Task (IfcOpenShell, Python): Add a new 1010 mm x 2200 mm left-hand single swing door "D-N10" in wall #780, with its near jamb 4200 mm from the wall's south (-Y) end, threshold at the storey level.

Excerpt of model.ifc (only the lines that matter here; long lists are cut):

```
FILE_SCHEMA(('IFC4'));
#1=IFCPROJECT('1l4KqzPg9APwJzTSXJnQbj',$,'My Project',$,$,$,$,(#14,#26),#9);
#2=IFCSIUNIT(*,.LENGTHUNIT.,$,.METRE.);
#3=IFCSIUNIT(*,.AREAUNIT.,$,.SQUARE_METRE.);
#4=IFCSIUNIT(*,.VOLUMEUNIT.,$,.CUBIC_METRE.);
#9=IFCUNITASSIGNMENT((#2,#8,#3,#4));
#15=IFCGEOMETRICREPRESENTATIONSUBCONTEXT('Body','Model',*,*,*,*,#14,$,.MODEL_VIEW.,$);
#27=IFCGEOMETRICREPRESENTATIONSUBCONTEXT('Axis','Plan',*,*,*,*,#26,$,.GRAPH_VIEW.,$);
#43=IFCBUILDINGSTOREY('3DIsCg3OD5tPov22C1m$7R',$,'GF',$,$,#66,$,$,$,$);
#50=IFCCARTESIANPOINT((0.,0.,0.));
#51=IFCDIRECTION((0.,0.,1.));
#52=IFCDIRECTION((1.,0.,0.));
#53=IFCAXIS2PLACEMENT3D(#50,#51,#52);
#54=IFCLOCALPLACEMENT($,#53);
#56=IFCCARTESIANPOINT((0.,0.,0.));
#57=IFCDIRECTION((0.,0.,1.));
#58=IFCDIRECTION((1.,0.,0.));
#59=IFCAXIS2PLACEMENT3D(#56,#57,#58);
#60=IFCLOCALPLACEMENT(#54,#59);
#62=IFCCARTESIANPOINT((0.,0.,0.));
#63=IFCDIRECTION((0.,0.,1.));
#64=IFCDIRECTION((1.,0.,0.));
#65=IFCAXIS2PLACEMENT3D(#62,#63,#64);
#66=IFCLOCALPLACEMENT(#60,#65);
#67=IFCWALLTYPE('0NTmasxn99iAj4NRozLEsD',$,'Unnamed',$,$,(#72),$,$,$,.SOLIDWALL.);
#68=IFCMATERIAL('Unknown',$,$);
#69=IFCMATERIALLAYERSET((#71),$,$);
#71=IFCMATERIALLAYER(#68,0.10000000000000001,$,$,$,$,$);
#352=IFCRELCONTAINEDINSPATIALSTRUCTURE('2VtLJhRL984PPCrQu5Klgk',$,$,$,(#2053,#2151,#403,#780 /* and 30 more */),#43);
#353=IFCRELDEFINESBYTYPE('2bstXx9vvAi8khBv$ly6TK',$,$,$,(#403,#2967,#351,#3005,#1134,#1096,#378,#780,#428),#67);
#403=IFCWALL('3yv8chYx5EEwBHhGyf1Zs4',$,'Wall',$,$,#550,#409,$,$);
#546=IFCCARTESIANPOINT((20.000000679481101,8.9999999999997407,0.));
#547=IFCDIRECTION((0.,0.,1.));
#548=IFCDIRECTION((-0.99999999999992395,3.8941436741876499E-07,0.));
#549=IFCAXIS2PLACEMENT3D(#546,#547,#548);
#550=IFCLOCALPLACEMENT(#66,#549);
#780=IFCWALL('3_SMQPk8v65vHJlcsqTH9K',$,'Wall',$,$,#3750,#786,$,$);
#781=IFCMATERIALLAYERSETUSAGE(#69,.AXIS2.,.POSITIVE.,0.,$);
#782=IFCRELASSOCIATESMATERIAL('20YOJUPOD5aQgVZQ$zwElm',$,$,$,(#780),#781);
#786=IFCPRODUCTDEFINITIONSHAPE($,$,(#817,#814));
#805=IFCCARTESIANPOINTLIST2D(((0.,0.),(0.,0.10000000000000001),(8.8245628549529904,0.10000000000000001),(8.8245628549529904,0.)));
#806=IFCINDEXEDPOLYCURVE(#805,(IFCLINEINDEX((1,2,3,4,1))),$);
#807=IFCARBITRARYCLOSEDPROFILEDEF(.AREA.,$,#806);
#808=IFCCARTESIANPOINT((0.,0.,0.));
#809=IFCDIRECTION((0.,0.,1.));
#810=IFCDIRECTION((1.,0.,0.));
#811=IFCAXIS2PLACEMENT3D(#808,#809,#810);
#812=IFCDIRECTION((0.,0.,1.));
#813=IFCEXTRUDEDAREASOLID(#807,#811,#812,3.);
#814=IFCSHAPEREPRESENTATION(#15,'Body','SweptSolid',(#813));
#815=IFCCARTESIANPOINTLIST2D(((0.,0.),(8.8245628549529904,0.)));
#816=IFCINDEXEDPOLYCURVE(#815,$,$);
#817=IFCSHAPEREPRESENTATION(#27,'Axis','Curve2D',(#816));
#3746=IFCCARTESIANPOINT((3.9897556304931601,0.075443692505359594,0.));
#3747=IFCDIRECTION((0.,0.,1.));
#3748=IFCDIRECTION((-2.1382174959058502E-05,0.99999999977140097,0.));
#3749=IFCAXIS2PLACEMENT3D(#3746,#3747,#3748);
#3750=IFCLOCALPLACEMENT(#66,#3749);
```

```python
import numpy as np
import ifcopenshell
import ifcopenshell.api.feature
import ifcopenshell.api.geometry
import ifcopenshell.api.root
import ifcopenshell.api.spatial
import ifcopenshell.geom
import ifcopenshell.util.element
import ifcopenshell.util.placement
import ifcopenshell.util.representation
import ifcopenshell.util.shape
import ifcopenshell.util.unit

model = ifcopenshell.open("model.ifc")
unit_scale = ifcopenshell.util.unit.calculate_unit_scale(model)
settings = ifcopenshell.geom.settings()


def volume(element):
    """Net volume in cubic metres, openings subtracted."""
    shape = ifcopenshell.geom.create_shape(settings, element)
    return ifcopenshell.util.shape.get_volume(shape.geometry)


wall = model.by_guid("3_SMQPk8v65vHJlcsqTH9K")
storey = ifcopenshell.util.element.get_container(wall, ifc_class="IfcBuildingStorey")
context = ifcopenshell.util.representation.get_context(model, "Model", "Body", "MODEL_VIEW")
before = volume(wall)

width, height, from_end, sill = 1.01, 2.2, 4.2, 0.0  # metres

# The wall runs along its own X axis, and the end named is its -X end.
wall_shape = ifcopenshell.geom.create_shape(settings, wall)
x, y, z = ifcopenshell.util.shape.get_vertices(wall_shape.geometry).T
start = x.min() + from_end
face, thickness = float(y.min()), float(y.max() - y.min())
wall_matrix = ifcopenshell.util.placement.get_local_placement(wall.ObjectPlacement)
level = ifcopenshell.util.placement.get_local_placement(storey.ObjectPlacement)[2, 3]


def in_wall(x, y):
    """Placement at x, y metres in the wall's axes, at sill height."""
    matrix = wall_matrix.copy()
    matrix[:, 3] = wall_matrix @ np.array([x / unit_scale, y / unit_scale, 0.0, 1.0])
    matrix[2, 3] = level + sill / unit_scale
    return matrix


# Opening: a box that overshoots both wall faces by 50 mm.
opening = ifcopenshell.api.root.create_entity(model, ifc_class="IfcOpeningElement", predefined_type="OPENING")
box = ifcopenshell.api.geometry.add_wall_representation(
    model, context=context, length=width, height=height, thickness=thickness + 0.1
)
ifcopenshell.api.geometry.assign_representation(model, product=opening, representation=box)
ifcopenshell.api.geometry.edit_object_placement(model, product=opening, matrix=in_wall(start, face - 0.05), is_si=False)
ifcopenshell.api.feature.add_feature(model, feature=opening, element=wall)

door = ifcopenshell.api.root.create_entity(model, ifc_class="IfcDoor", name="D-N10", predefined_type="DOOR")
door.OverallWidth, door.OverallHeight = width / unit_scale, height / unit_scale
door.OperationType = "SINGLE_SWING_LEFT"
body = ifcopenshell.api.geometry.add_door_representation(
    model,
    context=context,
    overall_width=door.OverallWidth,
    overall_height=door.OverallHeight,
    operation_type="SINGLE_SWING_LEFT",
    lining_properties={"LiningDepth": thickness / unit_scale, "ThresholdDepth": thickness / unit_scale},
)
ifcopenshell.api.geometry.assign_representation(model, product=door, representation=body)
ifcopenshell.api.spatial.assign_container(model, products=[door], relating_structure=storey)
ifcopenshell.api.feature.add_filling(model, opening=opening, element=door)

# The lining spans the wall, so the door starts at the wall face.
ifcopenshell.api.geometry.edit_object_placement(model, product=door, matrix=in_wall(start, face), is_si=False)

after = volume(wall)

print(f"wall volume {before:.3f} -> {after:.3f} m3")

model.write("model_edited.ifc")
```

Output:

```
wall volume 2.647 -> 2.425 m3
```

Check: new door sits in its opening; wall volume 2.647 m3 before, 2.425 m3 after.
